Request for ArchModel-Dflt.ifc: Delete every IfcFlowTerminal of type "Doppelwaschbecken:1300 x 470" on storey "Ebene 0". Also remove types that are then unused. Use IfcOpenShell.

First a look at what the model holds.

```python
import ifcopenshell
import ifcopenshell.util.element

model = ifcopenshell.open("ArchModel-Dflt.ifc")
print(model.schema)
storey = next(s for s in model.by_type("IfcBuildingStorey") if s.Name == "Ebene 0")
terminals = [e for e in ifcopenshell.util.element.get_decomposition(storey) if e.is_a("IfcFlowTerminal")]
seen = {}
for e in terminals:
    element_type = ifcopenshell.util.element.get_type(e)
    name = element_type.Name if element_type not in (None, e) else None
    seen[name] = seen.get(name, 0) + 1
for name, count in sorted(seen.items(), key=str):
    print(count, "x", name)
```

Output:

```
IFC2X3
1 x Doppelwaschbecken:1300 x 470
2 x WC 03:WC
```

```python
import ifcopenshell
import ifcopenshell.api.root
import ifcopenshell.util.element

model = ifcopenshell.open("ArchModel-Dflt.ifc")

storey = next(s for s in model.by_type("IfcBuildingStorey") if s.Name == "Ebene 0")
terminals = [e for e in ifcopenshell.util.element.get_decomposition(storey) if e.is_a("IfcFlowTerminal")]
targets = [e for e in terminals if (t := ifcopenshell.util.element.get_type(e)) not in (None, e) and t.Name == "Doppelwaschbecken:1300 x 470"]
types = {ifcopenshell.util.element.get_type(e) for e in targets} - {None, *targets}

for e in targets:
    ifcopenshell.api.root.remove_product(model, product=e)
print(len(targets), "removed")

unused = [t for t in types if not ifcopenshell.util.element.get_types(t)]
for t in unused:
    ifcopenshell.api.root.remove_product(model, product=t)
print(len(unused), "unused types removed")

model.write("ArchModel-Dflt_edited.ifc")
```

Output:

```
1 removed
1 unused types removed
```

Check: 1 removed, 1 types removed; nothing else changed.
